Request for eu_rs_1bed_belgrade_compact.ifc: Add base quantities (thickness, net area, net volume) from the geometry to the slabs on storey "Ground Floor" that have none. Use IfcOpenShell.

First a look at what the model holds.

```python
import ifcopenshell
import ifcopenshell.util.element
import ifcopenshell.util.unit

model = ifcopenshell.open("eu_rs_1bed_belgrade_compact.ifc")
print(model.schema)
for unit_type in ("LENGTHUNIT", "AREAUNIT", "VOLUMEUNIT"):
    print(unit_type, ifcopenshell.util.unit.calculate_unit_scale(model, unit_type))
storey = next(s for s in model.by_type("IfcBuildingStorey") if s.Name == "Ground Floor")
slabs = [e for e in ifcopenshell.util.element.get_decomposition(storey) if e.is_a("IfcSlab")]
for e in sorted(slabs, key=lambda e: e.id()):
    print(e.id(), e.is_a(), e.Name, list(ifcopenshell.util.element.get_psets(e, qtos_only=True)), sep=" | ")
```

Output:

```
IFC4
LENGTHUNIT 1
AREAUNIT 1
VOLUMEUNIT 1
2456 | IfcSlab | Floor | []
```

```python
import ifcopenshell
import ifcopenshell.api.pset
import ifcopenshell.geom
import ifcopenshell.util.element
import ifcopenshell.util.shape
import ifcopenshell.util.unit

model = ifcopenshell.open("eu_rs_1bed_belgrade_compact.ifc")
unit_scale = ifcopenshell.util.unit.calculate_unit_scale(model)
area_scale = ifcopenshell.util.unit.calculate_unit_scale(model, "AREAUNIT")
volume_scale = ifcopenshell.util.unit.calculate_unit_scale(model, "VOLUMEUNIT")
settings = ifcopenshell.geom.settings()

storey = next(s for s in model.by_type("IfcBuildingStorey") if s.Name == "Ground Floor")
slabs = [e for e in ifcopenshell.util.element.get_decomposition(storey) if e.is_a("IfcSlab")]

for e in sorted(slabs, key=lambda e: e.id()):
    if ifcopenshell.util.element.get_psets(e, qtos_only=True, should_inherit=False):
        continue
    # Geometry comes back in metres, in the element's own axes.
    shape = ifcopenshell.geom.create_shape(settings, e)
    values = {
        "Width": ifcopenshell.util.shape.get_z(shape.geometry) / unit_scale,
        "NetArea": ifcopenshell.util.shape.get_footprint_area(shape.geometry) / area_scale,
        "NetVolume": ifcopenshell.util.shape.get_volume(shape.geometry) / volume_scale,
    }
    qto = ifcopenshell.api.pset.add_qto(model, product=e, name="Qto_SlabBaseQuantities")
    ifcopenshell.api.pset.edit_qto(model, qto=qto, properties=values)
    print(e.id(), {k: round(v, 3) for k, v in values.items()})

model.write("eu_rs_1bed_belgrade_compact-out.ifc")
```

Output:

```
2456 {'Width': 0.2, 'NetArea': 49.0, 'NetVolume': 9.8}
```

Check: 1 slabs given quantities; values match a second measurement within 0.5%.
